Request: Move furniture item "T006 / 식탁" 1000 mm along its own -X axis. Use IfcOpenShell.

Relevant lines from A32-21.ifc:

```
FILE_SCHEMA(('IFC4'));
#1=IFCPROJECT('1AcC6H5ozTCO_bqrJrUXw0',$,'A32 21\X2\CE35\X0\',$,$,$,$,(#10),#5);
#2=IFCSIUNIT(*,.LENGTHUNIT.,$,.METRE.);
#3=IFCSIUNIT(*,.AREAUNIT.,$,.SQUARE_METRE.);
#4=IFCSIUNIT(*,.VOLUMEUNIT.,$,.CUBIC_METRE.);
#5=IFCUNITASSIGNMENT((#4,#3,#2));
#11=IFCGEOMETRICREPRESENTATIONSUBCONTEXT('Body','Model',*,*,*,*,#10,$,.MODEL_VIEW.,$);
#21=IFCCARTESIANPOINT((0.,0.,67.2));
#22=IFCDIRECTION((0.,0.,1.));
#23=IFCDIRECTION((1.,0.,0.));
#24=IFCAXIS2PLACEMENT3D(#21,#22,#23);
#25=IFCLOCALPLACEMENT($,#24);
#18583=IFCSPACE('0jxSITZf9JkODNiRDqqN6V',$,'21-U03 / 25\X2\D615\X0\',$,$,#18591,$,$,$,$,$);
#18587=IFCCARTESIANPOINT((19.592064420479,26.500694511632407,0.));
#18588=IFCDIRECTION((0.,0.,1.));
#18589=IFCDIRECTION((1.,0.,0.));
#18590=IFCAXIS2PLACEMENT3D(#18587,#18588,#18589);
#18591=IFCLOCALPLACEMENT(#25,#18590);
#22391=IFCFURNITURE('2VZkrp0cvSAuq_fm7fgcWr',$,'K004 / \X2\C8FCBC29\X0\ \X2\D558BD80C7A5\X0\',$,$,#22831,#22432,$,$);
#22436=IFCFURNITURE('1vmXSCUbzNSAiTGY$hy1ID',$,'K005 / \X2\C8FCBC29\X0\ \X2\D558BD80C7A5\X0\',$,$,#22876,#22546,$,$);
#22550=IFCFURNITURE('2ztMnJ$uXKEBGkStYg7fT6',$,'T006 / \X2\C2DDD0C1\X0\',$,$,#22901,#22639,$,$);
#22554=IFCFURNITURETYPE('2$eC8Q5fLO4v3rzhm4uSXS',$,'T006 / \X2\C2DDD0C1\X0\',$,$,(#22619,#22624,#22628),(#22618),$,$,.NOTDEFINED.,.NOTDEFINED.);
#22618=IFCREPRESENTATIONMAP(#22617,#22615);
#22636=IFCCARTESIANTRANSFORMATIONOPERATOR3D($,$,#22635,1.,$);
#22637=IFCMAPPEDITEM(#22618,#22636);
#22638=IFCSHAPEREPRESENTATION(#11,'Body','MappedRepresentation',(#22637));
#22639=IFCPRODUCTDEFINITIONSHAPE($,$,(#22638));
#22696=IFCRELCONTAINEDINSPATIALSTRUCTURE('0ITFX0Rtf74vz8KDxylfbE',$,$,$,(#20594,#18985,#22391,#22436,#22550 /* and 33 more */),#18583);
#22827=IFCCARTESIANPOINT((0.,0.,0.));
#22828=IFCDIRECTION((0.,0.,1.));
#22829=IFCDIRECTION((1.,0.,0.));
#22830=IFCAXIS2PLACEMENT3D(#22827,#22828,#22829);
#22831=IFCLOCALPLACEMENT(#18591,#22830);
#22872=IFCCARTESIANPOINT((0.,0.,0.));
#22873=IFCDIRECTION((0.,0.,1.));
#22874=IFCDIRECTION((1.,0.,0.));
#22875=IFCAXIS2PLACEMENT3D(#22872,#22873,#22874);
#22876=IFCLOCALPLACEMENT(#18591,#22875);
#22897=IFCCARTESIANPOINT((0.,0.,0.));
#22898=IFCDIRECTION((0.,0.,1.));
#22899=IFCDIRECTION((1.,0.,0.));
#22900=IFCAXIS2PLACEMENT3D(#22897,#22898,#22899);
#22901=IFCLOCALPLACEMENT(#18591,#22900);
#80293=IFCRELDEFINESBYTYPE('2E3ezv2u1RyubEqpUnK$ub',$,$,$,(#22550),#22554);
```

```python
import ifcopenshell
import ifcopenshell.api.geometry
import ifcopenshell.util.placement
import ifcopenshell.util.unit

model = ifcopenshell.open("A32-21.ifc")
unit_scale = ifcopenshell.util.unit.calculate_unit_scale(model)

item = model.by_guid("2ztMnJ$uXKEBGkStYg7fT6")
matrix = ifcopenshell.util.placement.get_local_placement(item.ObjectPlacement)
matrix[:3, 3] -= matrix[:3, 0] * 1 / unit_scale
ifcopenshell.api.geometry.edit_object_placement(model, product=item, matrix=matrix, is_si=False)

print(ifcopenshell.util.placement.get_local_placement(item.ObjectPlacement).round(3) + 0.0)

model.write("A32-21_updated.ifc")
```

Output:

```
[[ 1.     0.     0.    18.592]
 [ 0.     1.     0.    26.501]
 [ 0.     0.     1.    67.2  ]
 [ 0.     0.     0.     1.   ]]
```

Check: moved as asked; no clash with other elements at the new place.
